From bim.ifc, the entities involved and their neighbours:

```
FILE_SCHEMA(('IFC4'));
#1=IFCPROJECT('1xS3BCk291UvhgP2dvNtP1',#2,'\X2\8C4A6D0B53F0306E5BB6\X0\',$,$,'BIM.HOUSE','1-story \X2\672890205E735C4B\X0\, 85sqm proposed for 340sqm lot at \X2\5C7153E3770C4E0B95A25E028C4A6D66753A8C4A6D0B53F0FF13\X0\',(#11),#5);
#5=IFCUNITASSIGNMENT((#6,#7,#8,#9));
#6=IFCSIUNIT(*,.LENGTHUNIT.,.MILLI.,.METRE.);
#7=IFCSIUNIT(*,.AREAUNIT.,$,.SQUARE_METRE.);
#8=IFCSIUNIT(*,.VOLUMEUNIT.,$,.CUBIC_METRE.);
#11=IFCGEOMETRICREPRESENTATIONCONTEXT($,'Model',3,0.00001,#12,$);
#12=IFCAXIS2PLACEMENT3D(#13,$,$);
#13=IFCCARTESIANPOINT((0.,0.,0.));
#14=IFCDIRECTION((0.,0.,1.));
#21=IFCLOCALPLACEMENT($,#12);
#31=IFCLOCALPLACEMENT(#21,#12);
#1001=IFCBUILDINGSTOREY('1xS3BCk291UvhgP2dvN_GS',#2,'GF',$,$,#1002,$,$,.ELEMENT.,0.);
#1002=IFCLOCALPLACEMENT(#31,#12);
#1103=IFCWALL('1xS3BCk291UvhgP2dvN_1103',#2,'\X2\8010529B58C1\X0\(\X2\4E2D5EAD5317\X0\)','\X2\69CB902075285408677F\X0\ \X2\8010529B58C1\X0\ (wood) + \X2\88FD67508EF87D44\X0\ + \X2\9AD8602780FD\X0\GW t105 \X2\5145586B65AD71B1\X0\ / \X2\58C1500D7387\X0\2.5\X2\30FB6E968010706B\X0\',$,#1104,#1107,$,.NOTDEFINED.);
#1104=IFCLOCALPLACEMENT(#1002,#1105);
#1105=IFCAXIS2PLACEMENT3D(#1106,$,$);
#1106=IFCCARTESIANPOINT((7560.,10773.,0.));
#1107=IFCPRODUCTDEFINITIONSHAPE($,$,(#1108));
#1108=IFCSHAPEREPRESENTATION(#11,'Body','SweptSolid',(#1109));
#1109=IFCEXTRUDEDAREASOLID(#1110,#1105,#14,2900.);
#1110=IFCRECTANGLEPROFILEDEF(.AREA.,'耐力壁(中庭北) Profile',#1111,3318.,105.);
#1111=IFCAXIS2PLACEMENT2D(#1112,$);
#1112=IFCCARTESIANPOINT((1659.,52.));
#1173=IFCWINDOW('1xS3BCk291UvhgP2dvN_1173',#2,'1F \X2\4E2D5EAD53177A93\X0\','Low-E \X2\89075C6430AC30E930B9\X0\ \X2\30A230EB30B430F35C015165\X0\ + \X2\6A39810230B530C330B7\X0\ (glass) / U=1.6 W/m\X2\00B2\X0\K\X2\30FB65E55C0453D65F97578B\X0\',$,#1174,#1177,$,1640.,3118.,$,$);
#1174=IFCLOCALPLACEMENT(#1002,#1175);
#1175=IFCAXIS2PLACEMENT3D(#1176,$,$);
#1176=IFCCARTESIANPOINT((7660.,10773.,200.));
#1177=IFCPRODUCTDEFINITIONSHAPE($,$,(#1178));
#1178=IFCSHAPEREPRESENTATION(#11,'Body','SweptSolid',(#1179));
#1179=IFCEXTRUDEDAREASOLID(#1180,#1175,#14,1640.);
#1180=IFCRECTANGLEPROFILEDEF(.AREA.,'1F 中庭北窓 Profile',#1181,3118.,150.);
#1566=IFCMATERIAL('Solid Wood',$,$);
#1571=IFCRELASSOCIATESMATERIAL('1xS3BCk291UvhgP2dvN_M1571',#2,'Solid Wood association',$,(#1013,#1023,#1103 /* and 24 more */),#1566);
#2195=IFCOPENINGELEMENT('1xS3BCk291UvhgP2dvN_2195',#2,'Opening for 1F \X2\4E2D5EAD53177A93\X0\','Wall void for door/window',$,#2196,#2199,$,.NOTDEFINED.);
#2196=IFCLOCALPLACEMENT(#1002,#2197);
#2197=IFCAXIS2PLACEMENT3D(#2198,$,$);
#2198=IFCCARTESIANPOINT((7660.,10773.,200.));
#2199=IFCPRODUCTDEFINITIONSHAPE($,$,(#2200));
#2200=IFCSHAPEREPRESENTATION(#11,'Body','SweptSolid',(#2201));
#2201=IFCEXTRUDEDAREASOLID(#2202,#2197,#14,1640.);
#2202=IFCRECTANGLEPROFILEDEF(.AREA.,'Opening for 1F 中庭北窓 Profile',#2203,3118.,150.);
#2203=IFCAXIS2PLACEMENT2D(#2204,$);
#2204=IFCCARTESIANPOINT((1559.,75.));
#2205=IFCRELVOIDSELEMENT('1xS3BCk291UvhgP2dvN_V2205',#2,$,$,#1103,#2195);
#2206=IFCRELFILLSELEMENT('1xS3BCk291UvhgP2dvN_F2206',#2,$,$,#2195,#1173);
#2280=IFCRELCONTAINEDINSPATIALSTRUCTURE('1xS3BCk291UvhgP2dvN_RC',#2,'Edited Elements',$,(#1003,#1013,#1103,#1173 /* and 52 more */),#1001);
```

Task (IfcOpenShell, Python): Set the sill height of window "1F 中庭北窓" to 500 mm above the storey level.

```python
import numpy as np
import ifcopenshell
import ifcopenshell.api.geometry
import ifcopenshell.geom
import ifcopenshell.util.element
import ifcopenshell.util.placement
import ifcopenshell.util.shape
import ifcopenshell.util.unit

model = ifcopenshell.open("bim.ifc")
unit_scale = ifcopenshell.util.unit.calculate_unit_scale(model)

window = model.by_id(1173)
opening = window.FillsVoids[0].RelatingOpeningElement
storey = ifcopenshell.util.element.get_container(window, ifc_class="IfcBuildingStorey")
level = ifcopenshell.util.placement.get_local_placement(storey.ObjectPlacement)[2, 3]

# The opening's origin need not be at the sill, so measure its lowest point.
shape = ifcopenshell.geom.create_shape(ifcopenshell.geom.settings(), opening)
bottom = ifcopenshell.util.shape.get_shape_bottom_elevation(shape, shape.geometry) / unit_scale
dz = level + 0.5 / unit_scale - bottom

shift = np.array([0.0, 0.0, dz])
# The window is not placed relative to its opening, so move both.
for product in (opening, window):
    matrix = ifcopenshell.util.placement.get_local_placement(product.ObjectPlacement)
    matrix[:3, 3] += shift
    ifcopenshell.api.geometry.edit_object_placement(model, product=product, matrix=matrix, is_si=False)

print(f"moved by {dz * unit_scale:+.3f} m")

model.write("bim-out.ifc")
```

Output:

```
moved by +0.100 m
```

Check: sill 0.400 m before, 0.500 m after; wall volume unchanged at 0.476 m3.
